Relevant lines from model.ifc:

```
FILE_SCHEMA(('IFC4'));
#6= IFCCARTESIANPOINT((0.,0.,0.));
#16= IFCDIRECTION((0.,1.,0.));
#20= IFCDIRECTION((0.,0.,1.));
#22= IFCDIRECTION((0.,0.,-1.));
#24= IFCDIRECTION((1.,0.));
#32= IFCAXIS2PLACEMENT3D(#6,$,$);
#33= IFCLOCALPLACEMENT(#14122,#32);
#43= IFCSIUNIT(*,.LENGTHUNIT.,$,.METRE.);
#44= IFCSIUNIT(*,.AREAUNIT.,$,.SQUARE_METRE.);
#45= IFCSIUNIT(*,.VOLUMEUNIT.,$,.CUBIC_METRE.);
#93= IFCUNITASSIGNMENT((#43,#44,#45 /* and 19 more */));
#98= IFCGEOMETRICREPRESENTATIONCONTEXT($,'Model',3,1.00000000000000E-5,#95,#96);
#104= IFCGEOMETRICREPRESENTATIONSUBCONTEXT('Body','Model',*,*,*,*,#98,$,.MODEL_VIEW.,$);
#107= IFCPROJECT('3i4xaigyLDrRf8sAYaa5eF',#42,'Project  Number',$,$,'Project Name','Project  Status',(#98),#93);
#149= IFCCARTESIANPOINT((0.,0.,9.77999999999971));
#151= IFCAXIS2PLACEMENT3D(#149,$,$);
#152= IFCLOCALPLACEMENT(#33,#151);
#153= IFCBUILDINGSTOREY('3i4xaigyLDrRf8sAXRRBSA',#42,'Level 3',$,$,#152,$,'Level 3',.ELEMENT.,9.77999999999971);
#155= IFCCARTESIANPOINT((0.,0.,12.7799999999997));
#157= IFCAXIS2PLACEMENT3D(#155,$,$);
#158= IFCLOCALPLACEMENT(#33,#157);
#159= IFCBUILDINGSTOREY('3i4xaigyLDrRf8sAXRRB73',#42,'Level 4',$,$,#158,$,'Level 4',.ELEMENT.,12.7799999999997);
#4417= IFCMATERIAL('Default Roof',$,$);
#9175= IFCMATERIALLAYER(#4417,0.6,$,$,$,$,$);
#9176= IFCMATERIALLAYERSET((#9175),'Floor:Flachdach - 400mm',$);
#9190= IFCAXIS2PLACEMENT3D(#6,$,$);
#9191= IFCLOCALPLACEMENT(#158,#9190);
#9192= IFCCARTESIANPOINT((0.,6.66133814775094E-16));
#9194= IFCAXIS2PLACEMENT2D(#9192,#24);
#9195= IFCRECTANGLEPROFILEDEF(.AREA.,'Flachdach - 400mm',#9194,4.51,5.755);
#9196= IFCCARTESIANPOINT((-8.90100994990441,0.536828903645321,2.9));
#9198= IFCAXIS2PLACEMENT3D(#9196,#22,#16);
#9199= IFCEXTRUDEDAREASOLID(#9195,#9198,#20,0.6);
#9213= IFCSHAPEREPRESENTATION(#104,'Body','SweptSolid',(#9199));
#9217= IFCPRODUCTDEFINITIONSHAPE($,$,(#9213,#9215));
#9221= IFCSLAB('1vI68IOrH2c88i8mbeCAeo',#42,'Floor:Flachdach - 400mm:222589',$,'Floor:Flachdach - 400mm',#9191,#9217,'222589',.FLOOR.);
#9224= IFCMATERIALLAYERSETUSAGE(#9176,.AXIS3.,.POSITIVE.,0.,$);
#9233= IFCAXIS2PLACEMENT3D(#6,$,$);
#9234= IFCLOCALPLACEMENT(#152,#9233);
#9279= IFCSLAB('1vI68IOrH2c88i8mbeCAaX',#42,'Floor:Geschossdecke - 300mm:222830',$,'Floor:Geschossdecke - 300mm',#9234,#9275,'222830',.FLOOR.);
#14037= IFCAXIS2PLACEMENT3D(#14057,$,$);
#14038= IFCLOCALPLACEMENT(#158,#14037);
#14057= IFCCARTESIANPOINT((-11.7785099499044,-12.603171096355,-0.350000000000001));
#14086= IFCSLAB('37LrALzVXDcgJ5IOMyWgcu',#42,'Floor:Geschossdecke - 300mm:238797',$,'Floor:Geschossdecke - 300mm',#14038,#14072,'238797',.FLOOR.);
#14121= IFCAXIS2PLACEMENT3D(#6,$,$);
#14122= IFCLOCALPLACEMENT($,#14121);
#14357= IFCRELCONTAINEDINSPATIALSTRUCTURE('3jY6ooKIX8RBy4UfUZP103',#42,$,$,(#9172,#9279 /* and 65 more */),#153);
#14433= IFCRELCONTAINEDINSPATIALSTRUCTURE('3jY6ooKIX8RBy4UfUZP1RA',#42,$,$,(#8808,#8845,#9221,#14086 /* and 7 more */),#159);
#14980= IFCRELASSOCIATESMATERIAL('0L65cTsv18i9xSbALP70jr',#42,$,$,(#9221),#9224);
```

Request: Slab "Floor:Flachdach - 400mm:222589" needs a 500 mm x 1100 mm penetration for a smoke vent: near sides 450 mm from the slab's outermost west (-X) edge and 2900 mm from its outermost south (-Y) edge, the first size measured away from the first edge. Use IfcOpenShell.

```python
import numpy as np
import ifcopenshell
import ifcopenshell.api.feature
import ifcopenshell.api.geometry
import ifcopenshell.api.root
import ifcopenshell.geom
import ifcopenshell.util.placement
import ifcopenshell.util.representation
import ifcopenshell.util.shape
import ifcopenshell.util.unit

model = ifcopenshell.open("model.ifc")
unit_scale = ifcopenshell.util.unit.calculate_unit_scale(model)
settings = ifcopenshell.geom.settings()


def volume(element):
    """Net volume in cubic metres, openings subtracted."""
    shape = ifcopenshell.geom.create_shape(settings, element)
    return ifcopenshell.util.shape.get_volume(shape.geometry)


slab = model.by_guid("1vI68IOrH2c88i8mbeCAeo")
before = volume(slab)

# Extent in the slab's own axes, in metres. The edges named are its -X and -Y sides.
slab_shape = ifcopenshell.geom.create_shape(settings, slab)
vertices = ifcopenshell.util.shape.get_vertices(slab_shape.geometry)
x_min, y_min, bottom = vertices.min(axis=0)
top = vertices[:, 2].max()

opening = ifcopenshell.api.root.create_entity(model, ifc_class="IfcOpeningElement", name="Smoke vent opening", predefined_type="OPENING")
context = ifcopenshell.util.representation.get_context(model, "Model", "Body", "MODEL_VIEW")
width, depth = 0.5, 1.1
outline = [(0.0, 0.0), (width, 0.0), (width, depth), (0.0, depth), (0.0, 0.0)]
# Overshoot both faces by 50 mm so the cut is clean.
shape = ifcopenshell.api.geometry.add_slab_representation(
    model, context=context, depth=top - bottom + 0.1, polyline=outline
)
ifcopenshell.api.geometry.assign_representation(model, product=opening, representation=shape)

matrix = ifcopenshell.util.placement.get_local_placement(slab.ObjectPlacement)
matrix[:, 3] = matrix @ np.append(np.array([x_min + 0.45, y_min + 2.9, bottom - 0.05]) / unit_scale, 1.0)
ifcopenshell.api.geometry.edit_object_placement(model, product=opening, matrix=matrix, is_si=False)
ifcopenshell.api.feature.add_feature(model, feature=opening, element=slab)

after = volume(slab)

print(f"slab volume {before:.3f} -> {after:.3f} m3")

model.write("model-out.ifc")
```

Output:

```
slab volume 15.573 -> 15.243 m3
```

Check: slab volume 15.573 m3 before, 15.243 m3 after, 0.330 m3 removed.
